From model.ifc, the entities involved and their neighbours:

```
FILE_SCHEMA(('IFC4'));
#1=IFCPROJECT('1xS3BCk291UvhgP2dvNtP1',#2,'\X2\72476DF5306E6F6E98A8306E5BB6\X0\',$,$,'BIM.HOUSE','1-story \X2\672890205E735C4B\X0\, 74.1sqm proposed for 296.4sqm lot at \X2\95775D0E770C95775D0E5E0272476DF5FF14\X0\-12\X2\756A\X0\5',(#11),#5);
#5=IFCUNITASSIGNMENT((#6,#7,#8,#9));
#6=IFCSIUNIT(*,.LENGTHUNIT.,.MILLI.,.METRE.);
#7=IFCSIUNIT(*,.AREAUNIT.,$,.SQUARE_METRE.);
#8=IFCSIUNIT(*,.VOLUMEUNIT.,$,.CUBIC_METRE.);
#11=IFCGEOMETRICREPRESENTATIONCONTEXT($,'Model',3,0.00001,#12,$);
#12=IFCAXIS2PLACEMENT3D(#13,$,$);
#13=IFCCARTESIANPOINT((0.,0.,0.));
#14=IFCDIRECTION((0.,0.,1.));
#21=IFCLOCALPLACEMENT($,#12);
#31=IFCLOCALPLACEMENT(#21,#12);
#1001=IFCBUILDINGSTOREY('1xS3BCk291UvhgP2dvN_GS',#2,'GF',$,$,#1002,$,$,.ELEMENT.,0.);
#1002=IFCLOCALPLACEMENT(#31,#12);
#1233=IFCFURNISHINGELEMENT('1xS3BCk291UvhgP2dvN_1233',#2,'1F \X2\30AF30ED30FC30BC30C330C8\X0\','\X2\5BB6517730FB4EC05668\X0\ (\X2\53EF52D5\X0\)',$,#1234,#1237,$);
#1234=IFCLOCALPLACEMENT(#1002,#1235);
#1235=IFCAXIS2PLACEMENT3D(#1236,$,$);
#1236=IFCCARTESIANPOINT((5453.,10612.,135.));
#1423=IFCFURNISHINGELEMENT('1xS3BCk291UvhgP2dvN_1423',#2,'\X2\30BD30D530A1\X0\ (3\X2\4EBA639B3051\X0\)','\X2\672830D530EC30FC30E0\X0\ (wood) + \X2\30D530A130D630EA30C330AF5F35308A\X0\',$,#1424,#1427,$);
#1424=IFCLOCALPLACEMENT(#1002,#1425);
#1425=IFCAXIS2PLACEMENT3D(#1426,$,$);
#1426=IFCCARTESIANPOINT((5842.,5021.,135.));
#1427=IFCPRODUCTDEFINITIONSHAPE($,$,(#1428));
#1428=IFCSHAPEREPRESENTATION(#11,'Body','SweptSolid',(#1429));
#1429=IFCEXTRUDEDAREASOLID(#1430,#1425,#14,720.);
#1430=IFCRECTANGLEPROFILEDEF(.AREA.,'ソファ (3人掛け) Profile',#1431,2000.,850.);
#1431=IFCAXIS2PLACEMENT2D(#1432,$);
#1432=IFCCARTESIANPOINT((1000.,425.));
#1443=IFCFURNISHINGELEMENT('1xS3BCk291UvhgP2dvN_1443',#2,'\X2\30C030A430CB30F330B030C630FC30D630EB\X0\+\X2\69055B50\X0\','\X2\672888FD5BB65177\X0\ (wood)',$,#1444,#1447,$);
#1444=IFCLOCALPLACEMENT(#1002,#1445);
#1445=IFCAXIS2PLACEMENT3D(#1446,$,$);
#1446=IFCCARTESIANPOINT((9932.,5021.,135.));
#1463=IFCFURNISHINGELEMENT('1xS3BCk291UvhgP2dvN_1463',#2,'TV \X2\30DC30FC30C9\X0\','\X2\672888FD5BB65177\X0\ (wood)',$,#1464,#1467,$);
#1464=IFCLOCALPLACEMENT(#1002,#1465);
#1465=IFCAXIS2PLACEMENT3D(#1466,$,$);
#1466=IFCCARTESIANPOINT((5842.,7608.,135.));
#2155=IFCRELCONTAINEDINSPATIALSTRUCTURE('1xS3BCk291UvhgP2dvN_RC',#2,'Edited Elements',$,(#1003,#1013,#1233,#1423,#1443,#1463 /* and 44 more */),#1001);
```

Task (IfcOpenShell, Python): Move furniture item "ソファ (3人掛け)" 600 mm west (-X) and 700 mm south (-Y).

```python
import ifcopenshell
import ifcopenshell.api.geometry
import ifcopenshell.util.placement

model = ifcopenshell.open("model.ifc")

item = model.by_guid("1xS3BCk291UvhgP2dvN_1423")
matrix = ifcopenshell.util.placement.get_local_placement(item.ObjectPlacement)
matrix[0, 3] -= 600.0
matrix[1, 3] -= 700.0
ifcopenshell.api.geometry.edit_object_placement(model, product=item, matrix=matrix, is_si=False)

print(ifcopenshell.util.placement.get_local_placement(item.ObjectPlacement).round(3) + 0.0)

model.write("model_v2.ifc")
```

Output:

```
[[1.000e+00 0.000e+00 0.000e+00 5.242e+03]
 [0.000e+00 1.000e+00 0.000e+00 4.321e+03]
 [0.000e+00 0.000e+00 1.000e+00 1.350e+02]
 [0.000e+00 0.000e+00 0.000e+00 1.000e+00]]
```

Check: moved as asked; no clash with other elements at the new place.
